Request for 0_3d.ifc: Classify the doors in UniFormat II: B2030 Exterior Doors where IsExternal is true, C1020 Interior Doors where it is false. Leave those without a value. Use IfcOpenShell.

First a look at what the model holds.

```python
import ifcopenshell
import ifcopenshell.util.element

model = ifcopenshell.open("0_3d.ifc")
print(model.schema)
print("classifications:", [c.Name for c in model.by_type("IfcClassification")])
values = [ifcopenshell.util.element.get_pset(e, "Pset_DoorCommon", "IsExternal") for e in model.by_type("IfcDoor")]
for value in (True, False, None):
    print("IsExternal", value, values.count(value))
```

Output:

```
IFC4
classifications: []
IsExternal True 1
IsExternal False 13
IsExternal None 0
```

```python
import ifcopenshell
import ifcopenshell.api.classification
import ifcopenshell.util.element

model = ifcopenshell.open("0_3d.ifc")

system = ifcopenshell.api.classification.add_classification(model, classification="UniFormat II")

doors = model.by_type("IfcDoor")
external = {e: ifcopenshell.util.element.get_pset(e, "Pset_DoorCommon", "IsExternal") for e in doors}
for flag, code, name in ((True, "B2030", "Exterior Doors"), (False, "C1020", "Interior Doors")):
    products = [e for e in doors if external[e] is flag]
    ifcopenshell.api.classification.add_reference(
        model, products=products, classification=system, identification=code, name=name
    )
    print(code, len(products))

model.write("0_3d_rev.ifc")
```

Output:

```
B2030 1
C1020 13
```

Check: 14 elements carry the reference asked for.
